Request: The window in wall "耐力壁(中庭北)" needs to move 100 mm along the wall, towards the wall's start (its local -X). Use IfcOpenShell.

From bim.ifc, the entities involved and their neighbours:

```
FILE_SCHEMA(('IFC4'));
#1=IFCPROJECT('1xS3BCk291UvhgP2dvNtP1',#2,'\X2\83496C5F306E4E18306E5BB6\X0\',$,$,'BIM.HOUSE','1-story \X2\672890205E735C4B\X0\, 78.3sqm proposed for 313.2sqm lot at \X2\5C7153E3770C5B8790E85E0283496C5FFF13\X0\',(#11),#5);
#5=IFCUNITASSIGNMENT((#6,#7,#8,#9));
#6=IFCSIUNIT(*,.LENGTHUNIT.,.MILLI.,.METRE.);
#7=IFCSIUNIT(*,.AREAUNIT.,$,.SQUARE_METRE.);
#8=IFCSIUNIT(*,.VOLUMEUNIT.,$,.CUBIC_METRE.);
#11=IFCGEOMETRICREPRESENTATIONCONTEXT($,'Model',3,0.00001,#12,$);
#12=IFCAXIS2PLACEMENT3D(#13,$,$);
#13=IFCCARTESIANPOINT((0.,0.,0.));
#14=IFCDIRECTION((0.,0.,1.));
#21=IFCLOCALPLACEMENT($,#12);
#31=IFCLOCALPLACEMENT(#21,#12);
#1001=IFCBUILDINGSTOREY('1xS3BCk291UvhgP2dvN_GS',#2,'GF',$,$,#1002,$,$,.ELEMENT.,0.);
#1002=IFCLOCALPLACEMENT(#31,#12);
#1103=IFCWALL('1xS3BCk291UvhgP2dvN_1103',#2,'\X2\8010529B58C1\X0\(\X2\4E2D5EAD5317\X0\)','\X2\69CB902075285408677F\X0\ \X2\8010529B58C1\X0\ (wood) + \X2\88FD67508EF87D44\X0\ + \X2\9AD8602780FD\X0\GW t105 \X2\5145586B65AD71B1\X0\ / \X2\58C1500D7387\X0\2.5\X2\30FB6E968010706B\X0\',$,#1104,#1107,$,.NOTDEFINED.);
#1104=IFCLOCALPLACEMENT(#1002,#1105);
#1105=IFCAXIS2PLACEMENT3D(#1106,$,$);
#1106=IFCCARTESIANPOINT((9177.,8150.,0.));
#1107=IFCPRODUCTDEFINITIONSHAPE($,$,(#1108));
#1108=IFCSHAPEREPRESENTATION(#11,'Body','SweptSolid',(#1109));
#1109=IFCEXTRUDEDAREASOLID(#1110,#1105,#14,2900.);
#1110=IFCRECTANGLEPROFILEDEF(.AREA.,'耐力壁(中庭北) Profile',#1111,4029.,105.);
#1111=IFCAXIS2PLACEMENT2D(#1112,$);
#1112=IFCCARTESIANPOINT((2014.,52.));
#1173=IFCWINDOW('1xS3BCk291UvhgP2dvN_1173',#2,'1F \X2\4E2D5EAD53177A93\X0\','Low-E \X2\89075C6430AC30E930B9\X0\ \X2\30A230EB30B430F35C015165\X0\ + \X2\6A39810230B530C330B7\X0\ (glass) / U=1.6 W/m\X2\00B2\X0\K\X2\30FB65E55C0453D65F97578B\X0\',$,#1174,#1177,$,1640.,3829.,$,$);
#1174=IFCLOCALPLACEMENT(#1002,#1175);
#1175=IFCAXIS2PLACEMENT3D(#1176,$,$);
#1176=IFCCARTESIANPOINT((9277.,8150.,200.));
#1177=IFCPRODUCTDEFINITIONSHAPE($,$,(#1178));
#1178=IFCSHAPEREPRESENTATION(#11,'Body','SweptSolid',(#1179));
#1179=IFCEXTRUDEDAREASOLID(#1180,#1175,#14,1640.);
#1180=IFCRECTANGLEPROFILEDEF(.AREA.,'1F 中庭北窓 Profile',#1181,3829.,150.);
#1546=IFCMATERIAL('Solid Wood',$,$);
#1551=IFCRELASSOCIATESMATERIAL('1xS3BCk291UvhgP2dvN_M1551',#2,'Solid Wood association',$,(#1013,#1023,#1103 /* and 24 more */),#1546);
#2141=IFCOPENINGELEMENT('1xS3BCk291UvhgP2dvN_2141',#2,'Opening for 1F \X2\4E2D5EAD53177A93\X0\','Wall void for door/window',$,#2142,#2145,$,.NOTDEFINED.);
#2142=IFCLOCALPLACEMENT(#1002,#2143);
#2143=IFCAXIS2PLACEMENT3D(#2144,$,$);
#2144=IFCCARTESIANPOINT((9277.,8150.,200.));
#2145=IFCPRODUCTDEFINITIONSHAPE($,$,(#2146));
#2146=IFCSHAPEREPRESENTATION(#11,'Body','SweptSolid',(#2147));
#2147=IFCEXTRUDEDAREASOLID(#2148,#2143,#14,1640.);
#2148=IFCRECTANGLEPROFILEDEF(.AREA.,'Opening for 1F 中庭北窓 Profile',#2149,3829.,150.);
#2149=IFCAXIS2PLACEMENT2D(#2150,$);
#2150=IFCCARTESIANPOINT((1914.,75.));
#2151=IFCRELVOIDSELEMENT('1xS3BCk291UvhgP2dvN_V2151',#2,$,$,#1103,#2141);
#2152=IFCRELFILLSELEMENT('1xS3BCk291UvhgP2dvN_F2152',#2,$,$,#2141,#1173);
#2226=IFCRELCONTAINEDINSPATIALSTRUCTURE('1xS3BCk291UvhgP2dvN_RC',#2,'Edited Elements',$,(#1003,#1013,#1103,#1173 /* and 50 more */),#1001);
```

```python
import ifcopenshell
import ifcopenshell.api.geometry
import ifcopenshell.util.placement

model = ifcopenshell.open("bim.ifc")

window = model.by_guid("1xS3BCk291UvhgP2dvN_1173")
opening = window.FillsVoids[0].RelatingOpeningElement
wall = opening.VoidsElements[0].RelatingBuildingElement

wall_matrix = ifcopenshell.util.placement.get_local_placement(wall.ObjectPlacement)
shift = wall_matrix[:3, 0] * -100.0
before = ifcopenshell.util.placement.get_local_placement(window.ObjectPlacement)[:3, 3].copy()

# The window is not placed relative to its opening, so move both.
for product in (opening, window):
    matrix = ifcopenshell.util.placement.get_local_placement(product.ObjectPlacement)
    matrix[:3, 3] += shift
    ifcopenshell.api.geometry.edit_object_placement(model, product=product, matrix=matrix, is_si=False)

after = ifcopenshell.util.placement.get_local_placement(window.ObjectPlacement)[:3, 3]
print("window moved by", (after - before).round(3) + 0.0)

model.write("bim_edited.ifc")
```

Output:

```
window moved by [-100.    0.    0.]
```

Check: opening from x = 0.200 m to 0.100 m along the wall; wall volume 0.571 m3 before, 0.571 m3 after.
